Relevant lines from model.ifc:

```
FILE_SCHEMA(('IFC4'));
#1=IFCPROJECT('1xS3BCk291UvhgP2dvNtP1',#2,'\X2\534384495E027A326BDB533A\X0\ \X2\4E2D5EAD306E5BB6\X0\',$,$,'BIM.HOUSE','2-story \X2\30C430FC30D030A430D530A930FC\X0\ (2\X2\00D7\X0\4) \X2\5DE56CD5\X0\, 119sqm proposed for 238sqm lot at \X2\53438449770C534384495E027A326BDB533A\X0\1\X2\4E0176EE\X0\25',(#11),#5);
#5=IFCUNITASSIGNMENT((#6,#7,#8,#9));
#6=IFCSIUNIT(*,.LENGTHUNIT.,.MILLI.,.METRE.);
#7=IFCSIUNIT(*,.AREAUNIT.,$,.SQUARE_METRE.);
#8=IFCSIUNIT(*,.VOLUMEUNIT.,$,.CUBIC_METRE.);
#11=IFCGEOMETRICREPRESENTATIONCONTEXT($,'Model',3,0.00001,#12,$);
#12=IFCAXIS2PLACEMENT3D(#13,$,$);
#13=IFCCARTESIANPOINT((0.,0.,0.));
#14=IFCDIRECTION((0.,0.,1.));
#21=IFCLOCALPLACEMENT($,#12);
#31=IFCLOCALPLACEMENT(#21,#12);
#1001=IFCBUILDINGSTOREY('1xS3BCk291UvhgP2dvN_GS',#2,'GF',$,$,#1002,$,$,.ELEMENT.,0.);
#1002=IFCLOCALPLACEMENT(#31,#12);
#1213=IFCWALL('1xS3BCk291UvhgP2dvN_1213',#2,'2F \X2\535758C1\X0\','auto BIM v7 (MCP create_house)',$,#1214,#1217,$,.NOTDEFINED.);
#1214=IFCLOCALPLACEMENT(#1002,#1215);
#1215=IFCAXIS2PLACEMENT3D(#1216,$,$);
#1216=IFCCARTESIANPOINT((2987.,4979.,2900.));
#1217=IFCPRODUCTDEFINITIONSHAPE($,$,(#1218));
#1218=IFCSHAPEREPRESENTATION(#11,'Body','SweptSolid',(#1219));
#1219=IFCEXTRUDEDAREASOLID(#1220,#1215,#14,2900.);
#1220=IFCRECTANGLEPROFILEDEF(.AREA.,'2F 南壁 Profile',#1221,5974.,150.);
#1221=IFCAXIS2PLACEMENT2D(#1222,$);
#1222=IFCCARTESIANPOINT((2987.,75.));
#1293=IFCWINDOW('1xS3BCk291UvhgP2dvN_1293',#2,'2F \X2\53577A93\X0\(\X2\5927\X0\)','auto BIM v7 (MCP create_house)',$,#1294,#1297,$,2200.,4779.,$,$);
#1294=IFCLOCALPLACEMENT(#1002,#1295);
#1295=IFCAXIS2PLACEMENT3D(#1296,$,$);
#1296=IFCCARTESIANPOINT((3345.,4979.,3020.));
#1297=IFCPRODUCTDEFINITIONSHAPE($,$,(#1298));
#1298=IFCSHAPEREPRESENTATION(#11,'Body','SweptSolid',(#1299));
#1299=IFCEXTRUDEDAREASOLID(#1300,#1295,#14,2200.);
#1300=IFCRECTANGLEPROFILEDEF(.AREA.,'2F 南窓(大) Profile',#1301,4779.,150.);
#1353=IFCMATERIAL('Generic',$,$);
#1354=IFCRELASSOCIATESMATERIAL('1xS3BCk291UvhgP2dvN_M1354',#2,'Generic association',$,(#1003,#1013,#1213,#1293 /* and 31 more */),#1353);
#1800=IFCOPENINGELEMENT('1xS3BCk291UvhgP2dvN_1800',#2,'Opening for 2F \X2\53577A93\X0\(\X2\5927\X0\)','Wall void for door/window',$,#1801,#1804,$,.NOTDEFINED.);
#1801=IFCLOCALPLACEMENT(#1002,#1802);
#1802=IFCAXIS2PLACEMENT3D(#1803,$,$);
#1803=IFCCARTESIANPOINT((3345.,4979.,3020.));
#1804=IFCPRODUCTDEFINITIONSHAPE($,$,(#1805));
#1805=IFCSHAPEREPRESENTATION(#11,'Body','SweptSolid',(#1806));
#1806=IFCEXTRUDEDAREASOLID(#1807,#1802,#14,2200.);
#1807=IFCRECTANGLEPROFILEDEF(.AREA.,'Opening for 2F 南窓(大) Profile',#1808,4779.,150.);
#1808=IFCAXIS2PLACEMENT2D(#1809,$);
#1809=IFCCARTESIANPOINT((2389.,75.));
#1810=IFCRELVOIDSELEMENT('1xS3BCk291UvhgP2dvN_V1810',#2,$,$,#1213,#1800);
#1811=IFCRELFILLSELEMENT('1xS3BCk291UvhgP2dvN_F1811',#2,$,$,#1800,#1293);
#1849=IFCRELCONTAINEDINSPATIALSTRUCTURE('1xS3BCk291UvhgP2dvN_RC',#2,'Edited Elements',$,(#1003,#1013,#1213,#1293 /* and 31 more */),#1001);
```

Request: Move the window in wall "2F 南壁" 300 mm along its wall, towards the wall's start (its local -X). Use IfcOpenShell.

```python
import ifcopenshell
import ifcopenshell.api.geometry
import ifcopenshell.util.placement

model = ifcopenshell.open("model.ifc")

window = model.by_id(1293)
opening = window.FillsVoids[0].RelatingOpeningElement
wall = opening.VoidsElements[0].RelatingBuildingElement

wall_matrix = ifcopenshell.util.placement.get_local_placement(wall.ObjectPlacement)
shift = wall_matrix[:3, 0] * -300.0
before = ifcopenshell.util.placement.get_local_placement(window.ObjectPlacement)[:3, 3].copy()

# The window is not placed relative to its opening, so move both.
for product in (opening, window):
    matrix = ifcopenshell.util.placement.get_local_placement(product.ObjectPlacement)
    matrix[:3, 3] += shift
    ifcopenshell.api.geometry.edit_object_placement(model, product=product, matrix=matrix, is_si=False)

after = ifcopenshell.util.placement.get_local_placement(window.ObjectPlacement)[:3, 3]
print("window moved by", (after - before).round(3) + 0.0)

model.write("model_rev.ifc")
```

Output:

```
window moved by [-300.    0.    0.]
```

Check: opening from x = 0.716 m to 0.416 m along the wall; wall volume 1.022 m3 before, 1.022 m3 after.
